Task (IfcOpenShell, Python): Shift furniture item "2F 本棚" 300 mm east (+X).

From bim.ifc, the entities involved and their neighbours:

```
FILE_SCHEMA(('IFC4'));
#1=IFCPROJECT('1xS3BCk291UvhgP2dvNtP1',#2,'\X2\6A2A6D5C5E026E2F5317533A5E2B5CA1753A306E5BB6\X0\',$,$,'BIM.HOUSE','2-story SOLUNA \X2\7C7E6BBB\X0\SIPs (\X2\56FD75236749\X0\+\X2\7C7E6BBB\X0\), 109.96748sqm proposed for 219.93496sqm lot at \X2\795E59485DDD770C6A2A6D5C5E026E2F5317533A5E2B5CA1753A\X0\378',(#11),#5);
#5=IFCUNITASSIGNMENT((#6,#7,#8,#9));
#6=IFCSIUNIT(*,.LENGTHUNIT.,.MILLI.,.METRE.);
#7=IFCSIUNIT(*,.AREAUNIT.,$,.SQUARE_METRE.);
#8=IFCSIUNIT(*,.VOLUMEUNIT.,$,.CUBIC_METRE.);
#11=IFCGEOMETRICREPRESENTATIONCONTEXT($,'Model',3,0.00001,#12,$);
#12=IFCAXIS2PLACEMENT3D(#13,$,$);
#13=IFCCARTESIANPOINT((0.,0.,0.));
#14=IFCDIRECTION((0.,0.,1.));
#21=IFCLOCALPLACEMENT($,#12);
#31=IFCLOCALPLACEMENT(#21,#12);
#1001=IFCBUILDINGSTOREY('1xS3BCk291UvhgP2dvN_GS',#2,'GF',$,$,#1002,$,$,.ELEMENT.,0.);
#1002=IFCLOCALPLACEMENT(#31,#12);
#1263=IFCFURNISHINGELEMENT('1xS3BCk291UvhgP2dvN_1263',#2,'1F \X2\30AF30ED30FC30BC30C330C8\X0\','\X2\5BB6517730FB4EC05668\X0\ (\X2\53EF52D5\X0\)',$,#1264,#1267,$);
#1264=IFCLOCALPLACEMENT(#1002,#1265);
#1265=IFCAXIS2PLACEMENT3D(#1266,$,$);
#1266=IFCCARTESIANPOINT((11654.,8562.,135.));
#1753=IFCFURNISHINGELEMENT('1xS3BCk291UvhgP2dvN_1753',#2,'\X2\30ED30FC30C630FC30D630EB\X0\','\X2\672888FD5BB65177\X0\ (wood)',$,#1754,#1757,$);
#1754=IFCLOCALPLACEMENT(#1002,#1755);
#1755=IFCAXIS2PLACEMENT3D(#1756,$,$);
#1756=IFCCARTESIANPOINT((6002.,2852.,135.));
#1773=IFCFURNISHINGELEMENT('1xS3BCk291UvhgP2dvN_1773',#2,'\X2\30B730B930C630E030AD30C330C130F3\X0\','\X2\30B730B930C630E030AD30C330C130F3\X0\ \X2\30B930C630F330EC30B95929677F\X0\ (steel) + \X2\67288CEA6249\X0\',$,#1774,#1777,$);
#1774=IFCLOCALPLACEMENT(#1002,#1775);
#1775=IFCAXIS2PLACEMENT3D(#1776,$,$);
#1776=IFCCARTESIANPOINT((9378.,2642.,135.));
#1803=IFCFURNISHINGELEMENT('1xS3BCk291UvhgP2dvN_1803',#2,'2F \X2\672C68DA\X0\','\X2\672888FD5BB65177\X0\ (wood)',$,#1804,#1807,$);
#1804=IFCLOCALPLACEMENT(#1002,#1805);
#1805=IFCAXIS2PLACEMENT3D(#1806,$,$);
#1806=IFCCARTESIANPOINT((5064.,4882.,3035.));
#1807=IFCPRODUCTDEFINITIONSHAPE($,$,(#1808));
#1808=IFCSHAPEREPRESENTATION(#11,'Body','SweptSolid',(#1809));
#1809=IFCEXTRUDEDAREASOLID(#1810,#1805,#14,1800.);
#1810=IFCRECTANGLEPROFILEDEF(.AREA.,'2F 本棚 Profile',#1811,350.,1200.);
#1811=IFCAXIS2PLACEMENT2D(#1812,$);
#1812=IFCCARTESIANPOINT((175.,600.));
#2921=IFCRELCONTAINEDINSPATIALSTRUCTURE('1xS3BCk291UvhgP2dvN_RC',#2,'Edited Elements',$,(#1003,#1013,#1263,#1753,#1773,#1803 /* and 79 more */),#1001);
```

```python
import ifcopenshell
import ifcopenshell.api.geometry
import ifcopenshell.util.placement

model = ifcopenshell.open("bim.ifc")

item = model.by_id(1803)
matrix = ifcopenshell.util.placement.get_local_placement(item.ObjectPlacement)
matrix[0, 3] += 300.0
ifcopenshell.api.geometry.edit_object_placement(model, product=item, matrix=matrix, is_si=False)

print(ifcopenshell.util.placement.get_local_placement(item.ObjectPlacement).round(3) + 0.0)

model.write("bim-out.ifc")
```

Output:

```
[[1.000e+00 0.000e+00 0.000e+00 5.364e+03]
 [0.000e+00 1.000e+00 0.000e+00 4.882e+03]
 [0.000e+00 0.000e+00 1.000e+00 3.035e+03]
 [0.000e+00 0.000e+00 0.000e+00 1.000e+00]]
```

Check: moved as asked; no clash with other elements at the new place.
